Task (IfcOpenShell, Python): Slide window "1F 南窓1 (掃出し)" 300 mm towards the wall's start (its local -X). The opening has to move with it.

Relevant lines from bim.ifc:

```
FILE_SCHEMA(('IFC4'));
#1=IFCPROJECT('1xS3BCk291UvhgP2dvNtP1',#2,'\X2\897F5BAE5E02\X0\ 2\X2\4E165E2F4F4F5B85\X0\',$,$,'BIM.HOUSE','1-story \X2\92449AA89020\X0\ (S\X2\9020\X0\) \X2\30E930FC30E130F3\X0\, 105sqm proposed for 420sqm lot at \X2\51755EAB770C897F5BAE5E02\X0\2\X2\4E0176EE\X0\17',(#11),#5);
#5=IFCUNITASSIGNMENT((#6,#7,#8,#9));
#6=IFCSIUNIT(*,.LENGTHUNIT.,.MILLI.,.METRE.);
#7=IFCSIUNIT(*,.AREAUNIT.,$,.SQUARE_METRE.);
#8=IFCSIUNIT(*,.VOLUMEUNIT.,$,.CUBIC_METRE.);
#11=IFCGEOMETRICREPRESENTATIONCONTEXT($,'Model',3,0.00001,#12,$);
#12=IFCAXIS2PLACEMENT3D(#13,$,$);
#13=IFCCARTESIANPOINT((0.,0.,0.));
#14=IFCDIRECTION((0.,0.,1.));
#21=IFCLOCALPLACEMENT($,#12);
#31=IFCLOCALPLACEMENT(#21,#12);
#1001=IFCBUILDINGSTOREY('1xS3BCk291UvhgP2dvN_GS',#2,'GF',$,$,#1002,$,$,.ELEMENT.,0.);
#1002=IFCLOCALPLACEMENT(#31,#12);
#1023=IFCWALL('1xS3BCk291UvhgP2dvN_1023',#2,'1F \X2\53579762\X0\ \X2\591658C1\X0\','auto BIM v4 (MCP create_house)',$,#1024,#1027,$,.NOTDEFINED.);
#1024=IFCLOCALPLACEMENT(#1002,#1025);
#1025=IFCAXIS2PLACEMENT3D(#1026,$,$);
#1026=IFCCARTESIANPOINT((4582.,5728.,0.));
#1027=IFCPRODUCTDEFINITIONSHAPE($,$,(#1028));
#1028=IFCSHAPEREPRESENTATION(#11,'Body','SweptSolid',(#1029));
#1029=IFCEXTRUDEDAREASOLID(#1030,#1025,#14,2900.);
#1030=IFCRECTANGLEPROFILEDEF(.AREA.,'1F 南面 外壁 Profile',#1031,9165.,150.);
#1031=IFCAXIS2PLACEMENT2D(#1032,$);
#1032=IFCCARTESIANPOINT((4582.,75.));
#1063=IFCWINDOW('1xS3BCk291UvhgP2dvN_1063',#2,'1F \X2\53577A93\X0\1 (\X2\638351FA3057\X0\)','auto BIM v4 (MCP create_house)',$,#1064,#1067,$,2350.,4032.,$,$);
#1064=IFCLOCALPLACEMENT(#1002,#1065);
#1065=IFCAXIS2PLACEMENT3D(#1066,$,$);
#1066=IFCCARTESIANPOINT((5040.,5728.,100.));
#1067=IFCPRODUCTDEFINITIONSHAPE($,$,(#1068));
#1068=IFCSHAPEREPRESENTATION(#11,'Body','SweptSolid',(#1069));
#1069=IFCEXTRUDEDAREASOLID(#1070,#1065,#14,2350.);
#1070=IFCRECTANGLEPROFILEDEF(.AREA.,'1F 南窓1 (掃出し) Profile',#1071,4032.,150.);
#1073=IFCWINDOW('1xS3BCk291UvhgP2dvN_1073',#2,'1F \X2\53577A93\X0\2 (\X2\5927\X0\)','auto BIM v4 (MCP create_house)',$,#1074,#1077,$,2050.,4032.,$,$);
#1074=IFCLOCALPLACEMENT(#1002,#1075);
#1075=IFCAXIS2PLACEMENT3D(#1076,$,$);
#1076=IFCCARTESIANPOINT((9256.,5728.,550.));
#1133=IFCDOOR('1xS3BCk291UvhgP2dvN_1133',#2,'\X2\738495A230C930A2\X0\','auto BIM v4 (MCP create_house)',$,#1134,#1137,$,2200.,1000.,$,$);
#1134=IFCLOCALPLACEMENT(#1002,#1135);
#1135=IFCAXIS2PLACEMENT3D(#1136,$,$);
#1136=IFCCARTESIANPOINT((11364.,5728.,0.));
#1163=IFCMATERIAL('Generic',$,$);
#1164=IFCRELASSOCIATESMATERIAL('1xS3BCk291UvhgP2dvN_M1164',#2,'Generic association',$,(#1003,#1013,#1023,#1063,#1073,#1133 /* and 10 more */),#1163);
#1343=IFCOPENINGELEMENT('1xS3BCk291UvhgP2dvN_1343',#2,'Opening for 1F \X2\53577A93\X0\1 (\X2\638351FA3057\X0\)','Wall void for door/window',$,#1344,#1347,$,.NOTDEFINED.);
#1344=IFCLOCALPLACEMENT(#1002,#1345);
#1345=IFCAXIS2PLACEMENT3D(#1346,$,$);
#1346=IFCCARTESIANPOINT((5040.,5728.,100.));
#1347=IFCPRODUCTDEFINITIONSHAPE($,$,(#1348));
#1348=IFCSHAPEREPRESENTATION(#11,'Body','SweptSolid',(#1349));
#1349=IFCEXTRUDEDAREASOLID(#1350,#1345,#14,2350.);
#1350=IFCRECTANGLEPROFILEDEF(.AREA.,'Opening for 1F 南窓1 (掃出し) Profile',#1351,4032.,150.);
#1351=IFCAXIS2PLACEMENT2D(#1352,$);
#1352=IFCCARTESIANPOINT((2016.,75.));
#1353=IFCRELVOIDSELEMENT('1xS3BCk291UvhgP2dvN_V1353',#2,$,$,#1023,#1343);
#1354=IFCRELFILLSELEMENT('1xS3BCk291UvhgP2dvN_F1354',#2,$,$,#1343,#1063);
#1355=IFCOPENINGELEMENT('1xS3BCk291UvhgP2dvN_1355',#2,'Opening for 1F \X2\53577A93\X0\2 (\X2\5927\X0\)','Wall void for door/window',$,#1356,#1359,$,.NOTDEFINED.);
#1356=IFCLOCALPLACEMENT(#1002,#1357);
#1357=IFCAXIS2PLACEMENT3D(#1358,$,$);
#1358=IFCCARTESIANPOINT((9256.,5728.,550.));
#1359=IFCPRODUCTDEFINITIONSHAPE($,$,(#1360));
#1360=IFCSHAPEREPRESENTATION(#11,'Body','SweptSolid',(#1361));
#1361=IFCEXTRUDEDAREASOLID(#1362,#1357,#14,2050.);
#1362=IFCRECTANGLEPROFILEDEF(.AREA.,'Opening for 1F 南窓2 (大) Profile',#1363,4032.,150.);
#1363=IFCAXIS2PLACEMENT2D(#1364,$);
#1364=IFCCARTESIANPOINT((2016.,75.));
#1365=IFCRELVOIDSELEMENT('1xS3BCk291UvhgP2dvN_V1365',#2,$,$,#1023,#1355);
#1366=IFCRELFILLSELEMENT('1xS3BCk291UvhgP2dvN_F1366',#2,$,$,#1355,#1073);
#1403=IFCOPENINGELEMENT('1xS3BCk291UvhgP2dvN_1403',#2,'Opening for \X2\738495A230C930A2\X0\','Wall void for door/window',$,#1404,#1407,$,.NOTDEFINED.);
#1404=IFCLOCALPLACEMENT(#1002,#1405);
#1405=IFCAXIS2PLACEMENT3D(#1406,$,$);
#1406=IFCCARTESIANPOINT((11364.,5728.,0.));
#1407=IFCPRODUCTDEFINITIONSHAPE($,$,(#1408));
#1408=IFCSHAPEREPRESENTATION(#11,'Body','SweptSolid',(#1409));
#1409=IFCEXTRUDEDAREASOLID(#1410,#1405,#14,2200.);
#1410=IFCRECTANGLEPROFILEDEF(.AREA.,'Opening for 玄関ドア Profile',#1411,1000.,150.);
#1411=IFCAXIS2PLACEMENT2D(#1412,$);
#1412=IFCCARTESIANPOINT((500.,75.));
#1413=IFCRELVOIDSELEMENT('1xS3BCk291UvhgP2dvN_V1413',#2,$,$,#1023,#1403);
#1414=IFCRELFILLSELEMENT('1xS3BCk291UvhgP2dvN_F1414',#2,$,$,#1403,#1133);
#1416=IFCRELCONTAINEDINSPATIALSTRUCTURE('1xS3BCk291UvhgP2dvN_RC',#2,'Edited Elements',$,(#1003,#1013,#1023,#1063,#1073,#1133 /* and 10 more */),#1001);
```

```python
import ifcopenshell
import ifcopenshell.api.geometry
import ifcopenshell.util.placement
import ifcopenshell.util.unit

model = ifcopenshell.open("bim.ifc")
unit_scale = ifcopenshell.util.unit.calculate_unit_scale(model)

window = model.by_guid("1xS3BCk291UvhgP2dvN_1063")
opening = window.FillsVoids[0].RelatingOpeningElement
wall = opening.VoidsElements[0].RelatingBuildingElement

wall_matrix = ifcopenshell.util.placement.get_local_placement(wall.ObjectPlacement)
shift = wall_matrix[:3, 0] * -0.3 / unit_scale
before = ifcopenshell.util.placement.get_local_placement(window.ObjectPlacement)[:3, 3].copy()

# The window is not placed relative to its opening, so move both.
for product in (opening, window):
    matrix = ifcopenshell.util.placement.get_local_placement(product.ObjectPlacement)
    matrix[:3, 3] += shift
    ifcopenshell.api.geometry.edit_object_placement(model, product=product, matrix=matrix, is_si=False)

after = ifcopenshell.util.placement.get_local_placement(window.ObjectPlacement)[:3, 3]
print("window moved by", (after - before).round(3) + 0.0)

model.write("bim_updated.ifc")
```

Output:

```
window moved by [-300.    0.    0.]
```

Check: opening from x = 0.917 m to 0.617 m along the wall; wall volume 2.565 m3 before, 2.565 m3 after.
